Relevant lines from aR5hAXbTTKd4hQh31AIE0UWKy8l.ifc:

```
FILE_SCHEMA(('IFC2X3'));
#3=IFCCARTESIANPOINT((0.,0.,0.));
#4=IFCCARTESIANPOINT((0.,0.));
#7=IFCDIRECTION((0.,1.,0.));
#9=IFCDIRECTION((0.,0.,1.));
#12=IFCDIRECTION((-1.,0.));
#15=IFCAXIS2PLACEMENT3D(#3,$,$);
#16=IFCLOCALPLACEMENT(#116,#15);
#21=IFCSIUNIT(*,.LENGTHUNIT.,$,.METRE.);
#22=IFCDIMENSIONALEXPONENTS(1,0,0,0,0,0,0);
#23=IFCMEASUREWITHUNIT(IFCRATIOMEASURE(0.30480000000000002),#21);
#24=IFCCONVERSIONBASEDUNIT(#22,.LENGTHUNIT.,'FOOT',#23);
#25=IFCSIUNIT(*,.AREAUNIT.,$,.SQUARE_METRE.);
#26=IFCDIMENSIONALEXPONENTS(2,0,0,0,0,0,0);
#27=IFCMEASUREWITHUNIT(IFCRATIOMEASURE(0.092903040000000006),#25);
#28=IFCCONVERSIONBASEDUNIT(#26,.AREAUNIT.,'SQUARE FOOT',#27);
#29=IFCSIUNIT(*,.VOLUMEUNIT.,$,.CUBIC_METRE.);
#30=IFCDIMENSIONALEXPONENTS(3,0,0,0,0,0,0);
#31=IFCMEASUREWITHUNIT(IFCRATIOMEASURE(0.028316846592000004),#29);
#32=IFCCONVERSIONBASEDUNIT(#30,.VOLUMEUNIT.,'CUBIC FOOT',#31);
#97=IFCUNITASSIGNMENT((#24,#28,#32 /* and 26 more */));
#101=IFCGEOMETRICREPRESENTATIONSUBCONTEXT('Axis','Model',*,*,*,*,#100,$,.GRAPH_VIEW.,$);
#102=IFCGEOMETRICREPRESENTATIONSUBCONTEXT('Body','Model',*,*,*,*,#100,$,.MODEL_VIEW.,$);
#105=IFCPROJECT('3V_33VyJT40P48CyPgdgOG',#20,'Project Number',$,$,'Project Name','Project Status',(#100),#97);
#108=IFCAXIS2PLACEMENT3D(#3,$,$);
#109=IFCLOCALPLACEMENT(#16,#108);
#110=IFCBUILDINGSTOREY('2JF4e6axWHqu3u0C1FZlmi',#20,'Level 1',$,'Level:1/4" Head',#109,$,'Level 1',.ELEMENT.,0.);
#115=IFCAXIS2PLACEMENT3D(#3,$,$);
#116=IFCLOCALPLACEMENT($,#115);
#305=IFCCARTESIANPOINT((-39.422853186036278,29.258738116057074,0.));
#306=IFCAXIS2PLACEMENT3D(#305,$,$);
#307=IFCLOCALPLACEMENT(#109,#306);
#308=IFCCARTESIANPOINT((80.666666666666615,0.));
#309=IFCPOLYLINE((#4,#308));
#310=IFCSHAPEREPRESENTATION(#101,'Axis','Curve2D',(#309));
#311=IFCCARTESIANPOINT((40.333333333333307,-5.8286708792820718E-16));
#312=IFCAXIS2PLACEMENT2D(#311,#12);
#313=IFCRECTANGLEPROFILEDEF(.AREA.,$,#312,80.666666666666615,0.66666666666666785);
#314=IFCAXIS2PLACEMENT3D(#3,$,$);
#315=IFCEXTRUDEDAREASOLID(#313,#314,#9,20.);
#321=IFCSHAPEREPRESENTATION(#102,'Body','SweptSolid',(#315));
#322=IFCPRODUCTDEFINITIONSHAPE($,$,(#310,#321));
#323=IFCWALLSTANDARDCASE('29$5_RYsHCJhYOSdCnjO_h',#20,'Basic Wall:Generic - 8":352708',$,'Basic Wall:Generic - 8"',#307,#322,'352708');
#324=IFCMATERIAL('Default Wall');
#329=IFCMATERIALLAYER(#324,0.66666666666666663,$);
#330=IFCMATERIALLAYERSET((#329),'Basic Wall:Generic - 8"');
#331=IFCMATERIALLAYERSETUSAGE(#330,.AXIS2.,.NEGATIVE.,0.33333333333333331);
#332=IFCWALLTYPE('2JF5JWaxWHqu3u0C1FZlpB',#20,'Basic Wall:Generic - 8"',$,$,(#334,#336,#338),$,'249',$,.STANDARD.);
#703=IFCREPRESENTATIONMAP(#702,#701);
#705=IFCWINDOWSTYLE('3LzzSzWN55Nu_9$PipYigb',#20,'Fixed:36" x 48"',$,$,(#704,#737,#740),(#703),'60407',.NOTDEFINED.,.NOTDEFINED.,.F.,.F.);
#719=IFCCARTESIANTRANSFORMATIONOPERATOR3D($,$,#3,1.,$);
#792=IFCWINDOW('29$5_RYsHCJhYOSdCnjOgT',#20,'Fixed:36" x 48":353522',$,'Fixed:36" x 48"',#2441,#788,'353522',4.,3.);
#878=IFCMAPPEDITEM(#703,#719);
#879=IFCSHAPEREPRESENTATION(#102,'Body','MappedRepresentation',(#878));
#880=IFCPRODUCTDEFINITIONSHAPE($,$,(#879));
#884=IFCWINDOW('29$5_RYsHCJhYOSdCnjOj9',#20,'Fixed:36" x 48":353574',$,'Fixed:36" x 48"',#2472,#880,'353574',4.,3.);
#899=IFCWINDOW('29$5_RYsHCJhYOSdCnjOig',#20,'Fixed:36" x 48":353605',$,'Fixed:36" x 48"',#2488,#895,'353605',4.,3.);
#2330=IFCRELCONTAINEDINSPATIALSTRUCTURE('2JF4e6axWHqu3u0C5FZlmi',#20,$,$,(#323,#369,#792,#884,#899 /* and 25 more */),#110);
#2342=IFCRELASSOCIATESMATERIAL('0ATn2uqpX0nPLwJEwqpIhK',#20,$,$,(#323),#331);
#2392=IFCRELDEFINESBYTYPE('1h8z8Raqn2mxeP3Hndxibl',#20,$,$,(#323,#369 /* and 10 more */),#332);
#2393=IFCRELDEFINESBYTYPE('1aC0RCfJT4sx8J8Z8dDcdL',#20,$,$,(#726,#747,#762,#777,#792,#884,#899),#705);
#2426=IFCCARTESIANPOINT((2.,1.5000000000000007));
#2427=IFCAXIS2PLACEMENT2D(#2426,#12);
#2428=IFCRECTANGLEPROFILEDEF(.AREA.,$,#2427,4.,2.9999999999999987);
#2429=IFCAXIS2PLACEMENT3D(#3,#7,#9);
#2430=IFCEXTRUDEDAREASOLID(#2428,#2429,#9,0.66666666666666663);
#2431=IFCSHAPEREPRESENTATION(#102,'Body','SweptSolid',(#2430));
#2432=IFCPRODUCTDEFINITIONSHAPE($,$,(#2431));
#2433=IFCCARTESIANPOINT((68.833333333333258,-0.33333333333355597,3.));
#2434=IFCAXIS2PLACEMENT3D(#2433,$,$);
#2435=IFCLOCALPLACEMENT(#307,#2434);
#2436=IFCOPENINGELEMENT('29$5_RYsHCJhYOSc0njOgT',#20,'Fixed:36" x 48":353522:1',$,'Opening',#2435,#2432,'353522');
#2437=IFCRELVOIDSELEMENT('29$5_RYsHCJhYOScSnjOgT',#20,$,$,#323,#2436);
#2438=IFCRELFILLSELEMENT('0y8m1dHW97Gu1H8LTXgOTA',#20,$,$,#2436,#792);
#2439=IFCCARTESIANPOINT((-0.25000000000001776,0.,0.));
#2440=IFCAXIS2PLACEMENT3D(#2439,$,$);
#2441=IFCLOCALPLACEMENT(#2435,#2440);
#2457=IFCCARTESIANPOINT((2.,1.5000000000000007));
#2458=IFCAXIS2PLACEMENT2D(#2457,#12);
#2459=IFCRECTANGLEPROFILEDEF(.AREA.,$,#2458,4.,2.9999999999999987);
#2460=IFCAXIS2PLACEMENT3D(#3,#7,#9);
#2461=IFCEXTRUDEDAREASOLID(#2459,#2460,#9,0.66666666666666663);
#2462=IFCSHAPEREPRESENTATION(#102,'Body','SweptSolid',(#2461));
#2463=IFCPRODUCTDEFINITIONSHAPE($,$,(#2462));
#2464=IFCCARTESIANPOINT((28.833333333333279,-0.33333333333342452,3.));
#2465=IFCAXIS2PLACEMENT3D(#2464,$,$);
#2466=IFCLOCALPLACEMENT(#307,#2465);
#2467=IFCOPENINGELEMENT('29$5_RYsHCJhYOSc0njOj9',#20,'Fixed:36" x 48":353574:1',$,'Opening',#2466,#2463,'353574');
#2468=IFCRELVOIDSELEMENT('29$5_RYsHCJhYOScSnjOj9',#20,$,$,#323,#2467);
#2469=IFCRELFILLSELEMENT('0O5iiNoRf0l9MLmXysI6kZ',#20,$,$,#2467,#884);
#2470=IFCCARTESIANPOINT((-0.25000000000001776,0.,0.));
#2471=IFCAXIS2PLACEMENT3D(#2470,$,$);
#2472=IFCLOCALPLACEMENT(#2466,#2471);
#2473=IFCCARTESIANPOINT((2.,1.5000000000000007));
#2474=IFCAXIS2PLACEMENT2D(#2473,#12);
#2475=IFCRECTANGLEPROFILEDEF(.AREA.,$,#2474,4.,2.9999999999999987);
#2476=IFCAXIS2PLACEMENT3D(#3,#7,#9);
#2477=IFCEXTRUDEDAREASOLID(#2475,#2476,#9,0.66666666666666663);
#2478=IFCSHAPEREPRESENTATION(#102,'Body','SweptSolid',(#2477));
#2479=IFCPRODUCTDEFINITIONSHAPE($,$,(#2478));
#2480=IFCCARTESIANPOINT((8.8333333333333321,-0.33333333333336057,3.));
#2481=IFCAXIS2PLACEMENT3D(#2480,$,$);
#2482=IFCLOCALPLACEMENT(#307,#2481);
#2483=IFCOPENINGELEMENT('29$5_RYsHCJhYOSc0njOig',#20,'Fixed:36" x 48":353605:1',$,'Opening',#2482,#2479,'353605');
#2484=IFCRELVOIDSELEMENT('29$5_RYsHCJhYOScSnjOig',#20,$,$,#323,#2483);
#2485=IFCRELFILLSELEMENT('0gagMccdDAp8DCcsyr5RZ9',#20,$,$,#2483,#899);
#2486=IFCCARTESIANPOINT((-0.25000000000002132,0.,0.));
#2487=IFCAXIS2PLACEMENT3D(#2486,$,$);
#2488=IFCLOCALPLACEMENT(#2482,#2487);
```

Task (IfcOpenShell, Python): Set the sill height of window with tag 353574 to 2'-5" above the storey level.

```python
import numpy as np
import ifcopenshell
import ifcopenshell.api.geometry
import ifcopenshell.geom
import ifcopenshell.util.element
import ifcopenshell.util.placement
import ifcopenshell.util.shape
import ifcopenshell.util.unit

model = ifcopenshell.open("aR5hAXbTTKd4hQh31AIE0UWKy8l.ifc")
unit_scale = ifcopenshell.util.unit.calculate_unit_scale(model)

window = model.by_guid("29$5_RYsHCJhYOSdCnjOj9")
opening = window.FillsVoids[0].RelatingOpeningElement
storey = ifcopenshell.util.element.get_container(window, ifc_class="IfcBuildingStorey")
level = ifcopenshell.util.placement.get_local_placement(storey.ObjectPlacement)[2, 3]

# The opening's origin need not be at the sill, so measure its lowest point.
shape = ifcopenshell.geom.create_shape(ifcopenshell.geom.settings(), opening)
bottom = ifcopenshell.util.shape.get_shape_bottom_elevation(shape, shape.geometry) / unit_scale
dz = level + 29 * 0.0254 / unit_scale - bottom

shift = np.array([0.0, 0.0, dz])
# The window is placed relative to its opening, so it follows when the opening moves.
matrix = ifcopenshell.util.placement.get_local_placement(opening.ObjectPlacement)
matrix[:3, 3] += shift
ifcopenshell.api.geometry.edit_object_placement(
    model, product=opening, matrix=matrix, is_si=False, should_transform_children=True
)

print(f"moved by {dz * unit_scale:+.3f} m")

model.write("aR5hAXbTTKd4hQh31AIE0UWKy8l_updated.ifc")
```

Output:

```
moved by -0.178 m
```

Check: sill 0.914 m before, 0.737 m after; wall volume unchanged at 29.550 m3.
